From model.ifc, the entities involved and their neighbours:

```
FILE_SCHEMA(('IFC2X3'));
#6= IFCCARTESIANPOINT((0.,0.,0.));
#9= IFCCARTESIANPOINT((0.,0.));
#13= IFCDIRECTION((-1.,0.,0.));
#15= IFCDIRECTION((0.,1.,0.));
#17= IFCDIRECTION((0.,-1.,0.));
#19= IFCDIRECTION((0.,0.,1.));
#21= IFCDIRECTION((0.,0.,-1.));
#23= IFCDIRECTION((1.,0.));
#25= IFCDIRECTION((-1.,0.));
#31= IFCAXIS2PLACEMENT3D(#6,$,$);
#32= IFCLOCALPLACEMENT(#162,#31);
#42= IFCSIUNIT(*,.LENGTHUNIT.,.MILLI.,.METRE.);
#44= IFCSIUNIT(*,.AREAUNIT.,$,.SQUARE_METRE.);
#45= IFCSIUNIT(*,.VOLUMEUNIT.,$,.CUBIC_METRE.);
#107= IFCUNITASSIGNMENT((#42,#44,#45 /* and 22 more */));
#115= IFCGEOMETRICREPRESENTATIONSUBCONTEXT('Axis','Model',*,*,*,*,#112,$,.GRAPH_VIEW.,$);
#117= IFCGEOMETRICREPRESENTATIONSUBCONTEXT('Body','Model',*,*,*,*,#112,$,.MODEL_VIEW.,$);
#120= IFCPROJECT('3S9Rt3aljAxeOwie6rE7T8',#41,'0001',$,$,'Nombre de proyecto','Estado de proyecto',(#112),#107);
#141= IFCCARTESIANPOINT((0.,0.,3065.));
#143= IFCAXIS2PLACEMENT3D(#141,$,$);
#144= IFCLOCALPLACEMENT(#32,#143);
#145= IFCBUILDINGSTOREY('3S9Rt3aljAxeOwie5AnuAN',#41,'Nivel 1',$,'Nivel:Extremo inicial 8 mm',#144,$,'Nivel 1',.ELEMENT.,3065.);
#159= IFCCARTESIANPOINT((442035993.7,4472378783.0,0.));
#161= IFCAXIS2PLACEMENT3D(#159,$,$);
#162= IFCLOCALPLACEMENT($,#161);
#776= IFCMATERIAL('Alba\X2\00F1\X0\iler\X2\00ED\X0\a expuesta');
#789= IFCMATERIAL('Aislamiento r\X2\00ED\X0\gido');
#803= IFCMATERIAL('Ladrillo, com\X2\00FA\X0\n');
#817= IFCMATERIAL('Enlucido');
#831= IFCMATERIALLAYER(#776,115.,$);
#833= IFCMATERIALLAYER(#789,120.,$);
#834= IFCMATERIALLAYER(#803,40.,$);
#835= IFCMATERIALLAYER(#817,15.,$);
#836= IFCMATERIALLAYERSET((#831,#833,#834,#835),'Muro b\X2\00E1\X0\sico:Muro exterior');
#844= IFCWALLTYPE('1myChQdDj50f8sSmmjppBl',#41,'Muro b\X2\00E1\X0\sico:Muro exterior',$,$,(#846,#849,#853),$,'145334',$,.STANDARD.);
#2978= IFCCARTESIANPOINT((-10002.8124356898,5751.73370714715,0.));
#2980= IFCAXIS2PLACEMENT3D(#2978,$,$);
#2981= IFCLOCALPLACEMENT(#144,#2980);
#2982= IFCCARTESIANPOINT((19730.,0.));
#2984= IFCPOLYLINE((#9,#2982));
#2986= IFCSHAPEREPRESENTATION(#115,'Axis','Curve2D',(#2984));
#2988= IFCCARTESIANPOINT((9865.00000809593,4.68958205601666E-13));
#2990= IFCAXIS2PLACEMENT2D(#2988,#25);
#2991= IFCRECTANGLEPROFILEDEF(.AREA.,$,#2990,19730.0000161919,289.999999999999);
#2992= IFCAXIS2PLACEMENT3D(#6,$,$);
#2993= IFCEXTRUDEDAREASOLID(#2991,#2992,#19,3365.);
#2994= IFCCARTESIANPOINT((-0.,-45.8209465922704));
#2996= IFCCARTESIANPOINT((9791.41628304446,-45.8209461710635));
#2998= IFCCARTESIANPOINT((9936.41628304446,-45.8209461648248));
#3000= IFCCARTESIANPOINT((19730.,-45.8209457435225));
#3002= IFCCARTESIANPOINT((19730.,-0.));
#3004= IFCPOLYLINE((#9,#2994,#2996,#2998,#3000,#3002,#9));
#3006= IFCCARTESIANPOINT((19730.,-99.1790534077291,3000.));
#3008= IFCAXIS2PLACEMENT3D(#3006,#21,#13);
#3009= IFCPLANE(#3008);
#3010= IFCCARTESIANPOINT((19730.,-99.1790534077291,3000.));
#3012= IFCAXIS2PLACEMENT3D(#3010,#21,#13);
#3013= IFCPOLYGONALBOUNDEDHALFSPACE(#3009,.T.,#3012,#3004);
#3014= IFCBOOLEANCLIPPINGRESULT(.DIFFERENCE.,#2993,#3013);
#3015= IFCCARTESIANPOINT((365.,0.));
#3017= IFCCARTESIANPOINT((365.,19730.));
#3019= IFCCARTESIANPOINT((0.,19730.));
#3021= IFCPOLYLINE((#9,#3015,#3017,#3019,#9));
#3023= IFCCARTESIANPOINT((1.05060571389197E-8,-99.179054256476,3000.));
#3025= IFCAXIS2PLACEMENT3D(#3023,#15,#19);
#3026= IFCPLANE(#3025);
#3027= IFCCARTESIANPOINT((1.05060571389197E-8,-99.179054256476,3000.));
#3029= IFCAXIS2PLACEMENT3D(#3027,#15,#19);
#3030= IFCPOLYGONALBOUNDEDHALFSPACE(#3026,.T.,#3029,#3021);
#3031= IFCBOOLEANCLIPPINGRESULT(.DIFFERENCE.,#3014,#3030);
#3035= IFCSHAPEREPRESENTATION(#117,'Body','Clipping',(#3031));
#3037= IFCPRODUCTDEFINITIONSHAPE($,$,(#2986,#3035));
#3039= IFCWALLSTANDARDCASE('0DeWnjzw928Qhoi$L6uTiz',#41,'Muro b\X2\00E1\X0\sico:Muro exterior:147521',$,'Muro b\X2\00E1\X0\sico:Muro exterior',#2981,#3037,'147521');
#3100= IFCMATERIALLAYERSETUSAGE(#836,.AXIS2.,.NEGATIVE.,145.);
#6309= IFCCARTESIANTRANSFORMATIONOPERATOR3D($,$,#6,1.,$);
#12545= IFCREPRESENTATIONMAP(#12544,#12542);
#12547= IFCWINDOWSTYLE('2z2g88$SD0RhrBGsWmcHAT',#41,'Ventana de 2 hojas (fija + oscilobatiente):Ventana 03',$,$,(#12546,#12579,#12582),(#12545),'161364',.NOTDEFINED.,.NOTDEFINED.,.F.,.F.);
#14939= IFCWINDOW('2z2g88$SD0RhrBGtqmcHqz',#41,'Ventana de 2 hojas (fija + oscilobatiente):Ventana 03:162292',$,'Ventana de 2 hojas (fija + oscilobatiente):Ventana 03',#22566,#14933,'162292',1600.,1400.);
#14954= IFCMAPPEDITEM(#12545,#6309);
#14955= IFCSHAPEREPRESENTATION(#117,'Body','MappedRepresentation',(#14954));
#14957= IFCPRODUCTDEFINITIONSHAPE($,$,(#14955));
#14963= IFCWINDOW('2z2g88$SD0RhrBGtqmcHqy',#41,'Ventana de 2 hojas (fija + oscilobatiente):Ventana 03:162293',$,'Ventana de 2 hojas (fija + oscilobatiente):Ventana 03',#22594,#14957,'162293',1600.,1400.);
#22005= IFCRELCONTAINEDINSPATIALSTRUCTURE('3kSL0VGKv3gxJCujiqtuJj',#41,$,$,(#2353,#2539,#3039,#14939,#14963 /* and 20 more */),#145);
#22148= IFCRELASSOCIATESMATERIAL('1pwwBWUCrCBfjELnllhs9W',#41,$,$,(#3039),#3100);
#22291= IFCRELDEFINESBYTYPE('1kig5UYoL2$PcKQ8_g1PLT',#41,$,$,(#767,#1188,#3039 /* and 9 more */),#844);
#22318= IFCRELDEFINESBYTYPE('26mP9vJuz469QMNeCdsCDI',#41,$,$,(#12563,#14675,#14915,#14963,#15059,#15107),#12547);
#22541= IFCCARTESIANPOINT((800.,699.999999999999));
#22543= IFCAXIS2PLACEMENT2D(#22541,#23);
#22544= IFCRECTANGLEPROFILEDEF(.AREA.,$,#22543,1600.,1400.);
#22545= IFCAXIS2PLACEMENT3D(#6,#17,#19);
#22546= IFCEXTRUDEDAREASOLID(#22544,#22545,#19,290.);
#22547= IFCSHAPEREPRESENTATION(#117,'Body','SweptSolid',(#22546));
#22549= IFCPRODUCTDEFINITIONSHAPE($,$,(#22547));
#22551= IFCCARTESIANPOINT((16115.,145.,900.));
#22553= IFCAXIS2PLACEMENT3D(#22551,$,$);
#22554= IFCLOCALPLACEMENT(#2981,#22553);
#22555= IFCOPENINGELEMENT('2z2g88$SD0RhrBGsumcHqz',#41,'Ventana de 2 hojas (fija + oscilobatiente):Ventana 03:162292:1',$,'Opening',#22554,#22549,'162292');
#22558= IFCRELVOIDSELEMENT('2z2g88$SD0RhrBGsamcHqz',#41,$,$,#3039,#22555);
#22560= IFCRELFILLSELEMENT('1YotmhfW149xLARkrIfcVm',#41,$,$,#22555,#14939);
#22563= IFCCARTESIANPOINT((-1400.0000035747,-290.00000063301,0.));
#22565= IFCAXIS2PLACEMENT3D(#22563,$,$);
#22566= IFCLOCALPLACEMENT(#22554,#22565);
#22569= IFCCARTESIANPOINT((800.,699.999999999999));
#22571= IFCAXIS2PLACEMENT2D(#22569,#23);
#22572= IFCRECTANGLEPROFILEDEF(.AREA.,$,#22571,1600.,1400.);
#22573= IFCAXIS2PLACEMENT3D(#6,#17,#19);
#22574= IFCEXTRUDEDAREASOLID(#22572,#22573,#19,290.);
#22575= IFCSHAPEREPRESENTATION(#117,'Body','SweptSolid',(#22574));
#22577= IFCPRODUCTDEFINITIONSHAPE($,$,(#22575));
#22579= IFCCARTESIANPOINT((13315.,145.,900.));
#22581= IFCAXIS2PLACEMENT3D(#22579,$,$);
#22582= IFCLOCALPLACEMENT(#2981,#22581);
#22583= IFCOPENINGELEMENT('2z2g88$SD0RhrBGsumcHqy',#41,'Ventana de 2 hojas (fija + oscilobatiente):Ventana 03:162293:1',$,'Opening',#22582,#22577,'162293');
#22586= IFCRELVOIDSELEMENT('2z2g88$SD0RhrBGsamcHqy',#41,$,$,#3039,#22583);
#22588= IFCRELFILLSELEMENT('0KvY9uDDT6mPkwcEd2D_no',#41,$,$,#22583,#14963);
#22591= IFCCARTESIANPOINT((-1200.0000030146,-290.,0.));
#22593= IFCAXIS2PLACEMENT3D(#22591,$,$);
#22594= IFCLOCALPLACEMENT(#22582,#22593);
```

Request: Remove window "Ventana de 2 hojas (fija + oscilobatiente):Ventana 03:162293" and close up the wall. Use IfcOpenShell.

```python
import ifcopenshell
import ifcopenshell.api.feature
import ifcopenshell.api.root
import ifcopenshell.geom
import ifcopenshell.util.shape

model = ifcopenshell.open("model.ifc")
settings = ifcopenshell.geom.settings()


def volume(element):
    """Net volume in cubic metres, openings subtracted."""
    shape = ifcopenshell.geom.create_shape(settings, element)
    return ifcopenshell.util.shape.get_volume(shape.geometry)


window = model.by_guid("2z2g88$SD0RhrBGtqmcHqy")
opening = window.FillsVoids[0].RelatingOpeningElement
wall = opening.VoidsElements[0].RelatingBuildingElement
before = volume(wall)

ifcopenshell.api.root.remove_product(model, product=window)
ifcopenshell.api.feature.remove_feature(model, feature=opening)

after = volume(wall)

print(f"wall volume {before:.3f} -> {after:.3f} m3")

model.write("model-out.ifc")
```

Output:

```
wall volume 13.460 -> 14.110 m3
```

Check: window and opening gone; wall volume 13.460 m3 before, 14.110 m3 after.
